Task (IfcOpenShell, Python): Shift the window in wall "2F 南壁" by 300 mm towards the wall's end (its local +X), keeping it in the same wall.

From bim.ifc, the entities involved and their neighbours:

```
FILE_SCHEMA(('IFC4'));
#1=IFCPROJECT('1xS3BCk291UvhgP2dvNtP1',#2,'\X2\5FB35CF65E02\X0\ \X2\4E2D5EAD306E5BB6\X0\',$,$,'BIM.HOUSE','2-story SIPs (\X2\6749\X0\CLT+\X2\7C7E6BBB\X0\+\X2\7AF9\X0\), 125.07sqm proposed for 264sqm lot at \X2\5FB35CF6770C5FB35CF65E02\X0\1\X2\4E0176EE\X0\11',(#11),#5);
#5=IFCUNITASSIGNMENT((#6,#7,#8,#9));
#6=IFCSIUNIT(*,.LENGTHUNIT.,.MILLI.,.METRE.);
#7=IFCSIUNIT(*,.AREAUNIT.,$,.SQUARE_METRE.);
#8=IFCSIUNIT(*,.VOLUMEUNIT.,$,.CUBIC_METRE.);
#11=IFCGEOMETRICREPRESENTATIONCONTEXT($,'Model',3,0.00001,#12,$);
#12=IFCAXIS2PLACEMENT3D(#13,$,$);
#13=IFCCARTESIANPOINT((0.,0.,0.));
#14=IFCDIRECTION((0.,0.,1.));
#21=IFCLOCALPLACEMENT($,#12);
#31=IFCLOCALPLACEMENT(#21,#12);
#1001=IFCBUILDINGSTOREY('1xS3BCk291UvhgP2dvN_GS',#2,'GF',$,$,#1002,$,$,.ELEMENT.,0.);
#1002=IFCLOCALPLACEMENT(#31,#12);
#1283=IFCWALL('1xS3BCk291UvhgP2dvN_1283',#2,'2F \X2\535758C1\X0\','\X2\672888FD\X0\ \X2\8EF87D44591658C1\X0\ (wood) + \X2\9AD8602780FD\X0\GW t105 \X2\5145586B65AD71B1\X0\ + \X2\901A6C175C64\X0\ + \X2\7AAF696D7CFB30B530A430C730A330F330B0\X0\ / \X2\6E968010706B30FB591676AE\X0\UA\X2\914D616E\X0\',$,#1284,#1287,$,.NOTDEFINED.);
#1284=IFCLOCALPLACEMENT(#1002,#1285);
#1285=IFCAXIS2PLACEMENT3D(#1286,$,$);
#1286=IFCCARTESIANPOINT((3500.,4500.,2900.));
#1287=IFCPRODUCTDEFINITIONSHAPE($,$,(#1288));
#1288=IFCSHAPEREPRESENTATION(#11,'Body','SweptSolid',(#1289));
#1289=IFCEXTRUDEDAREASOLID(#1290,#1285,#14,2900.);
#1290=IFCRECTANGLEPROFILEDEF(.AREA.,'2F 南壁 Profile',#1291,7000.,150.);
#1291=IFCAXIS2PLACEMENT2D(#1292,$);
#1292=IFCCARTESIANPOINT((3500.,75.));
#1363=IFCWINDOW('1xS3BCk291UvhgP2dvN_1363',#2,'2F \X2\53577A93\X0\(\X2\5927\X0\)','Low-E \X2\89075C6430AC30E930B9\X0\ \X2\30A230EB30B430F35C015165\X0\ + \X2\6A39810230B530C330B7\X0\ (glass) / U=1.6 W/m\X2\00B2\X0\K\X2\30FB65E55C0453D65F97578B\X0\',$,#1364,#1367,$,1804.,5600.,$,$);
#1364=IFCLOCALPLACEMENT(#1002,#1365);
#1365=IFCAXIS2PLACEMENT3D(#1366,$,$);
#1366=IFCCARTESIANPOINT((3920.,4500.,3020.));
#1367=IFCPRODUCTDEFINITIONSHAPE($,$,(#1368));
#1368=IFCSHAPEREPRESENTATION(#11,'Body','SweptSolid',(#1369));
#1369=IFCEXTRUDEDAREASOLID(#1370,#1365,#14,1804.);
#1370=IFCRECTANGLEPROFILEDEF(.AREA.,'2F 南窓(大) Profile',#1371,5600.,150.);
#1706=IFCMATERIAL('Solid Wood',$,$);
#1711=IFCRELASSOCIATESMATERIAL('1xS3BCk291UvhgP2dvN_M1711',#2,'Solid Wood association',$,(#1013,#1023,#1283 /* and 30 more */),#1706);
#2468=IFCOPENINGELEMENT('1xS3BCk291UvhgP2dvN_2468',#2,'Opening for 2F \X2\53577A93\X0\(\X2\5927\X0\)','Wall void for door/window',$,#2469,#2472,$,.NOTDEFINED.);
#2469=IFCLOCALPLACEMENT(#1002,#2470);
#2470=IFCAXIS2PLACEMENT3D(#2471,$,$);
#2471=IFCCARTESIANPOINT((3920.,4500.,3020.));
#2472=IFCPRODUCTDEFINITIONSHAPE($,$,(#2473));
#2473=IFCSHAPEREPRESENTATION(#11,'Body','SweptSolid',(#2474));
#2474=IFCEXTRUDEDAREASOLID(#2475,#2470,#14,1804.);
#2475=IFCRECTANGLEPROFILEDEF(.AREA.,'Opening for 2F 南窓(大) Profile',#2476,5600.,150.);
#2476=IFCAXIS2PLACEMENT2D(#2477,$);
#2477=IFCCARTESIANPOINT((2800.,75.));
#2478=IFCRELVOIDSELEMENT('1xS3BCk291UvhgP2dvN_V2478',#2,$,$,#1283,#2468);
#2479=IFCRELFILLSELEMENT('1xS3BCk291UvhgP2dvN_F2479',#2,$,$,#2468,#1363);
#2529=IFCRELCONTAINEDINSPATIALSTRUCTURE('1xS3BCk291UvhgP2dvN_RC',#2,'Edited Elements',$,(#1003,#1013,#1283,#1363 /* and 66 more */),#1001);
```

```python
import ifcopenshell
import ifcopenshell.api.geometry
import ifcopenshell.util.placement
import ifcopenshell.util.unit

model = ifcopenshell.open("bim.ifc")
unit_scale = ifcopenshell.util.unit.calculate_unit_scale(model)

window = model.by_guid("1xS3BCk291UvhgP2dvN_1363")
opening = window.FillsVoids[0].RelatingOpeningElement
wall = opening.VoidsElements[0].RelatingBuildingElement

wall_matrix = ifcopenshell.util.placement.get_local_placement(wall.ObjectPlacement)
shift = wall_matrix[:3, 0] * 0.3 / unit_scale
before = ifcopenshell.util.placement.get_local_placement(window.ObjectPlacement)[:3, 3].copy()

# The window is not placed relative to its opening, so move both.
for product in (opening, window):
    matrix = ifcopenshell.util.placement.get_local_placement(product.ObjectPlacement)
    matrix[:3, 3] += shift
    ifcopenshell.api.geometry.edit_object_placement(model, product=product, matrix=matrix, is_si=False)

after = ifcopenshell.util.placement.get_local_placement(window.ObjectPlacement)[:3, 3]
print("window moved by", (after - before).round(3) + 0.0)

model.write("bim-out.ifc")
```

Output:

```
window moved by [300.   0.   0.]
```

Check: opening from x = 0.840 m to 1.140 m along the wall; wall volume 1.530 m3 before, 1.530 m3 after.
